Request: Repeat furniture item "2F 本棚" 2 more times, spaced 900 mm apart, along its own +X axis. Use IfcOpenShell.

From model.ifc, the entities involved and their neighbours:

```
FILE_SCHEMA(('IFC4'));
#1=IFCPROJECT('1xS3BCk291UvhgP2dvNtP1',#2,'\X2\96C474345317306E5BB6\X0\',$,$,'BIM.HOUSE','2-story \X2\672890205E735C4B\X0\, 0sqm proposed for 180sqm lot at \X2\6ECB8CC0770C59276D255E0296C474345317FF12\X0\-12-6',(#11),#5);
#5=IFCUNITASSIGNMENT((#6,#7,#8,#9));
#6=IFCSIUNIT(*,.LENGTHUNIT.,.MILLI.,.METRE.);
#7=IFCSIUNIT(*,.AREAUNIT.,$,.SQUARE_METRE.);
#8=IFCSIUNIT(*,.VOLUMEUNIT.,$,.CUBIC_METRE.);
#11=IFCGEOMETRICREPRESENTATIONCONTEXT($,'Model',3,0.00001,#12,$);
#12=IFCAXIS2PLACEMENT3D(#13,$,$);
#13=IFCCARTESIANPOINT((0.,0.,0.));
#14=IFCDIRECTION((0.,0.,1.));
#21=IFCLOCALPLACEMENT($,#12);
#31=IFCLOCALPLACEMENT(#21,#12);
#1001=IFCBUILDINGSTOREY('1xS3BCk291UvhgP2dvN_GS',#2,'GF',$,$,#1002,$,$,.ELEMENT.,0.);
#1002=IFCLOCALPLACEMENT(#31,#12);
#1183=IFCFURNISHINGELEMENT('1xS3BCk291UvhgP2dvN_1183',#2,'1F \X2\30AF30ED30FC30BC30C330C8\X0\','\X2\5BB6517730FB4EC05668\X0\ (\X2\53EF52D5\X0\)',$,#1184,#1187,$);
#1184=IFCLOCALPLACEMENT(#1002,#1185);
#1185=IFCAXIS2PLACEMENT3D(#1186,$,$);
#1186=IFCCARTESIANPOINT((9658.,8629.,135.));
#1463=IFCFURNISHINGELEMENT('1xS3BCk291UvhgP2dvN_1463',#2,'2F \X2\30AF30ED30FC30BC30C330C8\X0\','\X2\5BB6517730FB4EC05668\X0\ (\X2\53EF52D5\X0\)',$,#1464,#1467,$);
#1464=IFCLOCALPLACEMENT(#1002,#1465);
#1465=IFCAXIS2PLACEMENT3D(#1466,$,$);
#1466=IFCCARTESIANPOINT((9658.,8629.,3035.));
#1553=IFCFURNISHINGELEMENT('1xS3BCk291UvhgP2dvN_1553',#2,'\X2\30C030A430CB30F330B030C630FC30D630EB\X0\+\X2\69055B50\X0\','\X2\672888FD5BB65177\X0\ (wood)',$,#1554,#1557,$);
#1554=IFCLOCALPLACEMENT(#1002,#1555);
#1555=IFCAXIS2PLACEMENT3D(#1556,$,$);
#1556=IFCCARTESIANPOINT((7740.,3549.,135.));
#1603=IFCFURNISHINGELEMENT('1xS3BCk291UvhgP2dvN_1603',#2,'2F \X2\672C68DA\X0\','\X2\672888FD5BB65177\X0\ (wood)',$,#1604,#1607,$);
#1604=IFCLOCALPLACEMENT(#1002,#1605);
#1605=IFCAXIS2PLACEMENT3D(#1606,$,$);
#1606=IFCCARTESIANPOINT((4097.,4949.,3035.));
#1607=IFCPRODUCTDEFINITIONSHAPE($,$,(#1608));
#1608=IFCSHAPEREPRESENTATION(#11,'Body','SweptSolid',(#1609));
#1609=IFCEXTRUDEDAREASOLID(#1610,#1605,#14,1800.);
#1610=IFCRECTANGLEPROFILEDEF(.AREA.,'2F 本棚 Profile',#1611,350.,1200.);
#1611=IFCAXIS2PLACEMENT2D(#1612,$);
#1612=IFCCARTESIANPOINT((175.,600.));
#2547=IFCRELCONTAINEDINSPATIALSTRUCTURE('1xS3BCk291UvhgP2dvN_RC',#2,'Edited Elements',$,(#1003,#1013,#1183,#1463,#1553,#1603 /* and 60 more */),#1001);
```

```python
import ifcopenshell
import ifcopenshell.api.geometry
import ifcopenshell.api.root
import ifcopenshell.util.element
import ifcopenshell.util.placement
import ifcopenshell.util.unit

model = ifcopenshell.open("model.ifc")
unit_scale = ifcopenshell.util.unit.calculate_unit_scale(model)


def reuse_history(source, copy):
    """copy_class also copies each property set's owner history, people and application; keep the originals."""
    for rel in copy.IsDefinedBy:
        if rel.is_a("IfcRelDefinesByProperties") and (history := rel.RelatingPropertyDefinition.OwnerHistory):
            rel.RelatingPropertyDefinition.OwnerHistory = source.OwnerHistory
            ifcopenshell.util.element.remove_deep2(model, history)


source = model.by_guid("1xS3BCk291UvhgP2dvN_1603")
base = ifcopenshell.util.placement.get_local_placement(source.ObjectPlacement)
step = base[:3, 0] * 0.9 / unit_scale

for i in range(1, 3):
    copy = ifcopenshell.api.root.copy_class(model, product=source)
    copy.Representation = ifcopenshell.util.element.copy_deep(
        model, source.Representation, exclude=["IfcGeometricRepresentationContext", "IfcRepresentationMap"]
    )
    reuse_history(source, copy)
    matrix = base.copy()
    matrix[:3, 3] += i * step
    print("added at", matrix[:3, 3].round(3) + 0.0)
    ifcopenshell.api.geometry.edit_object_placement(model, product=copy, matrix=matrix, is_si=False)

model.write("model_rev.ifc")
```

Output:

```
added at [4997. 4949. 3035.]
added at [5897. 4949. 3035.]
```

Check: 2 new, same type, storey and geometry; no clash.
